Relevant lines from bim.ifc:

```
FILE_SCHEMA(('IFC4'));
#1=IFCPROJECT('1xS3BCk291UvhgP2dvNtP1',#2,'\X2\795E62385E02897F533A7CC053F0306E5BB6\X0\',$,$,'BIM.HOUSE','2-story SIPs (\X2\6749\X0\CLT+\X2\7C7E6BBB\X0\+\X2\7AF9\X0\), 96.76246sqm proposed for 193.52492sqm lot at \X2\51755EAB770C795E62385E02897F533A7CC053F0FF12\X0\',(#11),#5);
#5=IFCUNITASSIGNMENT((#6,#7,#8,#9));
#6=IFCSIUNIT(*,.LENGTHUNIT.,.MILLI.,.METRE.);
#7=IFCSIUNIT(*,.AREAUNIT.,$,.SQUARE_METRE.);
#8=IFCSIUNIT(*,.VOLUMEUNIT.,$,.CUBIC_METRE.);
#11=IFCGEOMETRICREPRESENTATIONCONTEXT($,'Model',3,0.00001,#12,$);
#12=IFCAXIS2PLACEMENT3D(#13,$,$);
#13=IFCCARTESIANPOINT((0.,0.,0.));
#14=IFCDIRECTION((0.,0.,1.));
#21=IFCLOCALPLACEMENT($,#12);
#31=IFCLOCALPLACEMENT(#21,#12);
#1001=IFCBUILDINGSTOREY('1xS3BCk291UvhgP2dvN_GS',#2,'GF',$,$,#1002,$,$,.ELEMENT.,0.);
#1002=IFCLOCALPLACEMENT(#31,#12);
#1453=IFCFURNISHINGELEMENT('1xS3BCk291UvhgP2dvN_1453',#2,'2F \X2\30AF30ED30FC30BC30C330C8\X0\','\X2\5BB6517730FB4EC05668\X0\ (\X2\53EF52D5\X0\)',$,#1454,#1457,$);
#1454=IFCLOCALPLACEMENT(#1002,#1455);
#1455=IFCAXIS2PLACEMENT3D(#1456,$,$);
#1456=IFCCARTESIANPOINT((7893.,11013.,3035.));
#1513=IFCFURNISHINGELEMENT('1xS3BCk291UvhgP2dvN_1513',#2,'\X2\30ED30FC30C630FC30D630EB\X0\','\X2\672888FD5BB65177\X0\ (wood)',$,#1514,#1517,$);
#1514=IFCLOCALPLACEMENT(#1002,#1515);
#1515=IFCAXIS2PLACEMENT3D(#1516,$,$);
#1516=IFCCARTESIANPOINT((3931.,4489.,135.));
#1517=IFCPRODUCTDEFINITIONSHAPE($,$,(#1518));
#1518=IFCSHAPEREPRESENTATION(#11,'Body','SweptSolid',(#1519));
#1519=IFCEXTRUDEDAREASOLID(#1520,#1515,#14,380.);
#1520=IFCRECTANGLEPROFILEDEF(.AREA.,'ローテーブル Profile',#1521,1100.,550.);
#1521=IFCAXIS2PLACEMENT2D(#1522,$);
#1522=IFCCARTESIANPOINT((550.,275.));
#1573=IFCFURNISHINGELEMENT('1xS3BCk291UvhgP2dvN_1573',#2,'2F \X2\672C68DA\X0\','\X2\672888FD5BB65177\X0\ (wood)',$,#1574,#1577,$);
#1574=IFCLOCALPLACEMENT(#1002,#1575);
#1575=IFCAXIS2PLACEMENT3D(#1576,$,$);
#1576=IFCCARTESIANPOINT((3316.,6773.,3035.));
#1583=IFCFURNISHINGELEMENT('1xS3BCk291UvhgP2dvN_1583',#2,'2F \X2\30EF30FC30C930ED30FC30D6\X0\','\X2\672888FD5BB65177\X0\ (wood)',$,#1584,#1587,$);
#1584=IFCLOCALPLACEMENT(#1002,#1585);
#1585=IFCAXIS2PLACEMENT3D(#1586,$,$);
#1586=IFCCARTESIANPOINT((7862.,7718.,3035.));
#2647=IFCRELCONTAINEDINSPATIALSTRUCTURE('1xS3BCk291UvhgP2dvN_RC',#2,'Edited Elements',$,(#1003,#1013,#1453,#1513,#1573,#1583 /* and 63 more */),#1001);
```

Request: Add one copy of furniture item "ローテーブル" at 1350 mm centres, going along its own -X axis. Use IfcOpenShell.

```python
import ifcopenshell
import ifcopenshell.api.geometry
import ifcopenshell.api.root
import ifcopenshell.util.element
import ifcopenshell.util.placement
import ifcopenshell.util.unit

model = ifcopenshell.open("bim.ifc")
unit_scale = ifcopenshell.util.unit.calculate_unit_scale(model)


def reuse_history(source, copy):
    """copy_class also copies each property set's owner history, people and application; keep the originals."""
    for rel in copy.IsDefinedBy:
        if rel.is_a("IfcRelDefinesByProperties") and (history := rel.RelatingPropertyDefinition.OwnerHistory):
            rel.RelatingPropertyDefinition.OwnerHistory = source.OwnerHistory
            ifcopenshell.util.element.remove_deep2(model, history)


source = model.by_guid("1xS3BCk291UvhgP2dvN_1513")
base = ifcopenshell.util.placement.get_local_placement(source.ObjectPlacement)
step = -base[:3, 0] * 1.35 / unit_scale

for i in range(1, 2):
    copy = ifcopenshell.api.root.copy_class(model, product=source)
    copy.Representation = ifcopenshell.util.element.copy_deep(
        model, source.Representation, exclude=["IfcGeometricRepresentationContext", "IfcRepresentationMap"]
    )
    reuse_history(source, copy)
    matrix = base.copy()
    matrix[:3, 3] += i * step
    print("added at", matrix[:3, 3].round(3) + 0.0)
    ifcopenshell.api.geometry.edit_object_placement(model, product=copy, matrix=matrix, is_si=False)

model.write("bim_edited.ifc")
```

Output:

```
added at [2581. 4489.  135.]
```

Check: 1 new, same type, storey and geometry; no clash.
